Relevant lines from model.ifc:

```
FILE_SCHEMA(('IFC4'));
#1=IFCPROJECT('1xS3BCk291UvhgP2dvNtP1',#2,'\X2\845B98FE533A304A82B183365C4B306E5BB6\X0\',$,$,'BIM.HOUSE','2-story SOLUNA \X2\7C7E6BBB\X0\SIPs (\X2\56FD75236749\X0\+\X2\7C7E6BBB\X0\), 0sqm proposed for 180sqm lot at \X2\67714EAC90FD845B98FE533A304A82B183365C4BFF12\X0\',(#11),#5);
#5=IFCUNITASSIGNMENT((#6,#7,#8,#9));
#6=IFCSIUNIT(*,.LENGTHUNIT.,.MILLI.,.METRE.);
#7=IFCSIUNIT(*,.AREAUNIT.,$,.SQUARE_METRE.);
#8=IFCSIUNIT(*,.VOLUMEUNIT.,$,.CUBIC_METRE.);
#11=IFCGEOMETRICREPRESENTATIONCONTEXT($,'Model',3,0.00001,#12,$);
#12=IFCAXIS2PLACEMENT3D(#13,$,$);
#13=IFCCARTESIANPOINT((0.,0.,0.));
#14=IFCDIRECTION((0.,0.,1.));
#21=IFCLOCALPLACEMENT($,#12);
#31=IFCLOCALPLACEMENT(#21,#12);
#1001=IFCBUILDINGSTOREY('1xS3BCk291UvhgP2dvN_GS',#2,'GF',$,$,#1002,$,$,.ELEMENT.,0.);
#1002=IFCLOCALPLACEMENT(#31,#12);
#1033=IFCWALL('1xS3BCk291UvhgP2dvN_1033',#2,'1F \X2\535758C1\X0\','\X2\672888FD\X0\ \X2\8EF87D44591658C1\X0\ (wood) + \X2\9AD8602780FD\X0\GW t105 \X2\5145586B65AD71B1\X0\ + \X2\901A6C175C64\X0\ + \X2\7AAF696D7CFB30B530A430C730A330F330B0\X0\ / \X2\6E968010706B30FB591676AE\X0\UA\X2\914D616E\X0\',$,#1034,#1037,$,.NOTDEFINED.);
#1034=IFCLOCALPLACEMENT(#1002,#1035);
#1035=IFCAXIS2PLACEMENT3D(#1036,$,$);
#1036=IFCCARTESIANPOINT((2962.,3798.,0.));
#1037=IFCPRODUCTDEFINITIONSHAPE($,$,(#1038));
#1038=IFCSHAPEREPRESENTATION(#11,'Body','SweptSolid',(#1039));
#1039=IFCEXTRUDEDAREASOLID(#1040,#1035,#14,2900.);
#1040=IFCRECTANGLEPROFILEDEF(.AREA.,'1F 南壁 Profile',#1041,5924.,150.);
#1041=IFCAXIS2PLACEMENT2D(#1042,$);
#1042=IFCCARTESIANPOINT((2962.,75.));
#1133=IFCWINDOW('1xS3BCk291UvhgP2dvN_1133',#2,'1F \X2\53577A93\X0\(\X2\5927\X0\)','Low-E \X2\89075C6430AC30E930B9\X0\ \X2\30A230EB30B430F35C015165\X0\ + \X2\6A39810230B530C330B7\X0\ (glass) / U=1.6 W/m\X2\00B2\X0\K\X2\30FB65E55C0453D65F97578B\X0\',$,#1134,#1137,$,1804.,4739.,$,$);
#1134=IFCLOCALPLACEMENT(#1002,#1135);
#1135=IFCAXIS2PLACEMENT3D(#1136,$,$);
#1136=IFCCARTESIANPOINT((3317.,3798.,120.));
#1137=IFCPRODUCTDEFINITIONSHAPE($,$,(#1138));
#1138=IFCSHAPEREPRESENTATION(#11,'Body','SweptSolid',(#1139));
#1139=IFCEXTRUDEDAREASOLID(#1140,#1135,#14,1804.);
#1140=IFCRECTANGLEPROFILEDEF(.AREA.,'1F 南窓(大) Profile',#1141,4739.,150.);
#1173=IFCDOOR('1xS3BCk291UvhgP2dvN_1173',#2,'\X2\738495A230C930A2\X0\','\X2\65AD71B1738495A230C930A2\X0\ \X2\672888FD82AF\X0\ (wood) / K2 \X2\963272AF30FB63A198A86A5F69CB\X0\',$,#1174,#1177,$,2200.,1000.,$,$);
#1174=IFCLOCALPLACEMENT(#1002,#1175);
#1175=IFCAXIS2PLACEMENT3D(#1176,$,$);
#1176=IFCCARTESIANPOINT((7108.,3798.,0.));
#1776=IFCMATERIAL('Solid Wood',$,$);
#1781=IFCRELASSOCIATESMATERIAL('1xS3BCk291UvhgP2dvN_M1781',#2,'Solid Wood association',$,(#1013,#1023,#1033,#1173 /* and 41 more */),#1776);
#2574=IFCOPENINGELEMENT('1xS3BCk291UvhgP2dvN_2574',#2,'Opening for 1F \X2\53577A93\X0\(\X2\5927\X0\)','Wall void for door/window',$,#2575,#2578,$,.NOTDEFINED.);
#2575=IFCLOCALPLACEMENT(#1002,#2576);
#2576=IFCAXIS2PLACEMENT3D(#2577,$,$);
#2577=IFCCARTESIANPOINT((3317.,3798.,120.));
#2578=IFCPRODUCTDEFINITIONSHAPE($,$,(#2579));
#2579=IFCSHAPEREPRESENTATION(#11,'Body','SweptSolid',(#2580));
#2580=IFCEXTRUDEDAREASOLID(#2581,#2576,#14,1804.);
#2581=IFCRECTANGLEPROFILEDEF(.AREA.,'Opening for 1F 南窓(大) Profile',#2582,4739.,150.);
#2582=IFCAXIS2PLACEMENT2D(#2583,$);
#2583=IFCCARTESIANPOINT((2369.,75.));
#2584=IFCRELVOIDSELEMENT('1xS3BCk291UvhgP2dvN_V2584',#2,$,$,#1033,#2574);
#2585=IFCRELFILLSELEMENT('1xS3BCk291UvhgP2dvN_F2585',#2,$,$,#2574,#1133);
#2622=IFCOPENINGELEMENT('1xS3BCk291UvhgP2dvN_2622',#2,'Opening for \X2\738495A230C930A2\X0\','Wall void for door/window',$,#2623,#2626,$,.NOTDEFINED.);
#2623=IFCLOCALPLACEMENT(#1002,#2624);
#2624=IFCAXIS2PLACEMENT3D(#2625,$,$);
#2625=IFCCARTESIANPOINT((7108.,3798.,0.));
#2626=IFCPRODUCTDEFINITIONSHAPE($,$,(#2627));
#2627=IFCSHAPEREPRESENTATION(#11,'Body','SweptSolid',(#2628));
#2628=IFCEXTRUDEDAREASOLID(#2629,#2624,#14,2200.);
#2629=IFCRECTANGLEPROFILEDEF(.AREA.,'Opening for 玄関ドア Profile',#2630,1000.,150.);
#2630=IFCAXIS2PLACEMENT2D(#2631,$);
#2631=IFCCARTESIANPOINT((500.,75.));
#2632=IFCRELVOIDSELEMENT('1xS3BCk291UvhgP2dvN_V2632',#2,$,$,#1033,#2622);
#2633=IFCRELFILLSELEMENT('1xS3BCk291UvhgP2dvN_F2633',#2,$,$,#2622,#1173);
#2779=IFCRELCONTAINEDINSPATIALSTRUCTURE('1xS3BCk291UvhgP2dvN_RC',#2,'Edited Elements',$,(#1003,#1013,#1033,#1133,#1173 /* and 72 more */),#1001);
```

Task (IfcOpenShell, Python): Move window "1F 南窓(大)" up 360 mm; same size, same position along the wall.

```python
import numpy as np
import ifcopenshell
import ifcopenshell.api.geometry
import ifcopenshell.util.placement
import ifcopenshell.util.unit

model = ifcopenshell.open("model.ifc")
unit_scale = ifcopenshell.util.unit.calculate_unit_scale(model)

window = model.by_guid("1xS3BCk291UvhgP2dvN_1133")
opening = window.FillsVoids[0].RelatingOpeningElement
dz = 0.36 / unit_scale

shift = np.array([0.0, 0.0, dz])
# The window is not placed relative to its opening, so move both.
for product in (opening, window):
    matrix = ifcopenshell.util.placement.get_local_placement(product.ObjectPlacement)
    matrix[:3, 3] += shift
    ifcopenshell.api.geometry.edit_object_placement(model, product=product, matrix=matrix, is_si=False)

print(f"moved by {dz * unit_scale:+.3f} m")

model.write("model-out.ifc")
```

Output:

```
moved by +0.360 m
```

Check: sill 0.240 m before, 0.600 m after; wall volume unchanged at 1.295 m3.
